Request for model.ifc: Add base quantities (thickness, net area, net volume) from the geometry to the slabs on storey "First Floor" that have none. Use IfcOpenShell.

First a look at what the model holds.

```python
import ifcopenshell
import ifcopenshell.util.element
import ifcopenshell.util.unit

model = ifcopenshell.open("model.ifc")
print(model.schema)
for unit_type in ("LENGTHUNIT", "AREAUNIT", "VOLUMEUNIT"):
    print(unit_type, ifcopenshell.util.unit.calculate_unit_scale(model, unit_type))
storey = next(s for s in model.by_type("IfcBuildingStorey") if s.Name == "First Floor")
slabs = [e for e in ifcopenshell.util.element.get_decomposition(storey) if e.is_a("IfcSlab")]
for e in sorted(slabs, key=lambda e: e.id()):
    print(e.id(), e.is_a(), e.Name, list(ifcopenshell.util.element.get_psets(e, qtos_only=True)), sep=" | ")
```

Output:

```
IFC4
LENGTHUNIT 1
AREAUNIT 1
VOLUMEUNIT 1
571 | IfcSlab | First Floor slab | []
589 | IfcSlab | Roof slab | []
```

```python
import ifcopenshell
import ifcopenshell.api.pset
import ifcopenshell.geom
import ifcopenshell.util.element
import ifcopenshell.util.shape
import ifcopenshell.util.unit

model = ifcopenshell.open("model.ifc")
unit_scale = ifcopenshell.util.unit.calculate_unit_scale(model)
area_scale = ifcopenshell.util.unit.calculate_unit_scale(model, "AREAUNIT")
volume_scale = ifcopenshell.util.unit.calculate_unit_scale(model, "VOLUMEUNIT")
settings = ifcopenshell.geom.settings()

storey = next(s for s in model.by_type("IfcBuildingStorey") if s.Name == "First Floor")
slabs = [e for e in ifcopenshell.util.element.get_decomposition(storey) if e.is_a("IfcSlab")]

for e in sorted(slabs, key=lambda e: e.id()):
    if ifcopenshell.util.element.get_psets(e, qtos_only=True, should_inherit=False):
        continue
    # Geometry comes back in metres, in the element's own axes.
    shape = ifcopenshell.geom.create_shape(settings, e)
    values = {
        "Width": ifcopenshell.util.shape.get_z(shape.geometry) / unit_scale,
        "NetArea": ifcopenshell.util.shape.get_footprint_area(shape.geometry) / area_scale,
        "NetVolume": ifcopenshell.util.shape.get_volume(shape.geometry) / volume_scale,
    }
    qto = ifcopenshell.api.pset.add_qto(model, product=e, name="Qto_SlabBaseQuantities")
    ifcopenshell.api.pset.edit_qto(model, qto=qto, properties=values)
    print(e.id(), {k: round(v, 3) for k, v in values.items()})

model.write("model-out.ifc")
```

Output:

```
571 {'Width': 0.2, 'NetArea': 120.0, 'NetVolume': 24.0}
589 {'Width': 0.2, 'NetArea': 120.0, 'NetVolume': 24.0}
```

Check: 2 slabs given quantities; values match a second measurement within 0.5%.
